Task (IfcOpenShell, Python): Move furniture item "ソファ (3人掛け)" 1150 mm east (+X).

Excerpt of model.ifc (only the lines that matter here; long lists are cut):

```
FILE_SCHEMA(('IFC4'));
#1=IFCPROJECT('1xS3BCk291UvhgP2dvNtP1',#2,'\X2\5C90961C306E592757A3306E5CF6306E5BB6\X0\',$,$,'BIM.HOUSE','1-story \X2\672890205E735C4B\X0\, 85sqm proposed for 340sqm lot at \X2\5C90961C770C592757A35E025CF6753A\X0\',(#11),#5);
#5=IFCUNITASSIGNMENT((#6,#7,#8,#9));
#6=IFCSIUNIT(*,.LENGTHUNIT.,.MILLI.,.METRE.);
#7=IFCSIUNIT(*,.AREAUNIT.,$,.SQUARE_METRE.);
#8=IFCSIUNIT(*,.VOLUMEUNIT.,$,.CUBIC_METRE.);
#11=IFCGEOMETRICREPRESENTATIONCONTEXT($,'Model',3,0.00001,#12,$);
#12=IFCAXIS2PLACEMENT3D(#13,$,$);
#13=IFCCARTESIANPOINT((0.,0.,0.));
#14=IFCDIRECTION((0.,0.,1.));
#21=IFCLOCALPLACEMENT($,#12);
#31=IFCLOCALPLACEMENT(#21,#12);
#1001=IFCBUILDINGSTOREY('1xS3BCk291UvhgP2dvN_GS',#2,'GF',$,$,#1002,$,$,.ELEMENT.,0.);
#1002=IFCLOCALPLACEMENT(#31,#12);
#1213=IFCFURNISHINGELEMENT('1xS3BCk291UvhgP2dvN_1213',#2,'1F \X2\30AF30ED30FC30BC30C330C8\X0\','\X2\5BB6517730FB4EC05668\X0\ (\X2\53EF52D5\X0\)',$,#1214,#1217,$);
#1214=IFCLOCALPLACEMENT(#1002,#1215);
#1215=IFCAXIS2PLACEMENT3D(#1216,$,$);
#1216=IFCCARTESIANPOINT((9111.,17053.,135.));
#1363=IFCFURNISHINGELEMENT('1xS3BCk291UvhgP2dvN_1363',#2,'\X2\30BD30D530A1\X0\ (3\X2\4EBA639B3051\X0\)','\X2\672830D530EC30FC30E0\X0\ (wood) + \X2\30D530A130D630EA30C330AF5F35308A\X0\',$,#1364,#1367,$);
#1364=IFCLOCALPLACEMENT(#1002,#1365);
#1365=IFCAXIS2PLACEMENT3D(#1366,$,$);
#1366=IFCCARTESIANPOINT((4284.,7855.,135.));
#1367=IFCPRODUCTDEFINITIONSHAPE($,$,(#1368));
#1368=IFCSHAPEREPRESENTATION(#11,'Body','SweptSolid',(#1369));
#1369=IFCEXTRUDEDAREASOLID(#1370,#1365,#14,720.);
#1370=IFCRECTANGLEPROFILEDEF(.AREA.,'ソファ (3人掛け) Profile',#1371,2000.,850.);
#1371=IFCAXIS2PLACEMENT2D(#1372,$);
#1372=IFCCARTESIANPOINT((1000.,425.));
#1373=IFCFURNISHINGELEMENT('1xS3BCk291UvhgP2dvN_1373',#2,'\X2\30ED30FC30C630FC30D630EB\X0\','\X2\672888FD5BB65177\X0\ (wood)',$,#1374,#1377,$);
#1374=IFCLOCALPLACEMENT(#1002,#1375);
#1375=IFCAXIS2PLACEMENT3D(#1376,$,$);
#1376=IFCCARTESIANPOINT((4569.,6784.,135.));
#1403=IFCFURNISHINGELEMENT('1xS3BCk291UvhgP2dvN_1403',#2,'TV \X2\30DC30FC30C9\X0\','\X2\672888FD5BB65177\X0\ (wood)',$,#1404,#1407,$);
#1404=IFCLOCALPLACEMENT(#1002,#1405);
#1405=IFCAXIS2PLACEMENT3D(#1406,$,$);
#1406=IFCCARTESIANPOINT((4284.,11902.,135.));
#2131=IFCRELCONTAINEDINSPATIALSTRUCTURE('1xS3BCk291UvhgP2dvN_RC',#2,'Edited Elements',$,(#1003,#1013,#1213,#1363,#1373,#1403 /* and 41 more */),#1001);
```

```python
import ifcopenshell
import ifcopenshell.api.geometry
import ifcopenshell.util.placement
import ifcopenshell.util.unit

model = ifcopenshell.open("model.ifc")
unit_scale = ifcopenshell.util.unit.calculate_unit_scale(model)

item = model.by_guid("1xS3BCk291UvhgP2dvN_1363")
matrix = ifcopenshell.util.placement.get_local_placement(item.ObjectPlacement)
matrix[0, 3] += 1.15 / unit_scale
ifcopenshell.api.geometry.edit_object_placement(model, product=item, matrix=matrix, is_si=False)

print(ifcopenshell.util.placement.get_local_placement(item.ObjectPlacement).round(3) + 0.0)

model.write("model_v2.ifc")
```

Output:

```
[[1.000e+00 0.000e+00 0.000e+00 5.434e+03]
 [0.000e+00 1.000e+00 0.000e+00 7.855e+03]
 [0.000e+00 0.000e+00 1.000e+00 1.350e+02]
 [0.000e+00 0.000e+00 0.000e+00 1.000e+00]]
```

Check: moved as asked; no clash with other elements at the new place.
